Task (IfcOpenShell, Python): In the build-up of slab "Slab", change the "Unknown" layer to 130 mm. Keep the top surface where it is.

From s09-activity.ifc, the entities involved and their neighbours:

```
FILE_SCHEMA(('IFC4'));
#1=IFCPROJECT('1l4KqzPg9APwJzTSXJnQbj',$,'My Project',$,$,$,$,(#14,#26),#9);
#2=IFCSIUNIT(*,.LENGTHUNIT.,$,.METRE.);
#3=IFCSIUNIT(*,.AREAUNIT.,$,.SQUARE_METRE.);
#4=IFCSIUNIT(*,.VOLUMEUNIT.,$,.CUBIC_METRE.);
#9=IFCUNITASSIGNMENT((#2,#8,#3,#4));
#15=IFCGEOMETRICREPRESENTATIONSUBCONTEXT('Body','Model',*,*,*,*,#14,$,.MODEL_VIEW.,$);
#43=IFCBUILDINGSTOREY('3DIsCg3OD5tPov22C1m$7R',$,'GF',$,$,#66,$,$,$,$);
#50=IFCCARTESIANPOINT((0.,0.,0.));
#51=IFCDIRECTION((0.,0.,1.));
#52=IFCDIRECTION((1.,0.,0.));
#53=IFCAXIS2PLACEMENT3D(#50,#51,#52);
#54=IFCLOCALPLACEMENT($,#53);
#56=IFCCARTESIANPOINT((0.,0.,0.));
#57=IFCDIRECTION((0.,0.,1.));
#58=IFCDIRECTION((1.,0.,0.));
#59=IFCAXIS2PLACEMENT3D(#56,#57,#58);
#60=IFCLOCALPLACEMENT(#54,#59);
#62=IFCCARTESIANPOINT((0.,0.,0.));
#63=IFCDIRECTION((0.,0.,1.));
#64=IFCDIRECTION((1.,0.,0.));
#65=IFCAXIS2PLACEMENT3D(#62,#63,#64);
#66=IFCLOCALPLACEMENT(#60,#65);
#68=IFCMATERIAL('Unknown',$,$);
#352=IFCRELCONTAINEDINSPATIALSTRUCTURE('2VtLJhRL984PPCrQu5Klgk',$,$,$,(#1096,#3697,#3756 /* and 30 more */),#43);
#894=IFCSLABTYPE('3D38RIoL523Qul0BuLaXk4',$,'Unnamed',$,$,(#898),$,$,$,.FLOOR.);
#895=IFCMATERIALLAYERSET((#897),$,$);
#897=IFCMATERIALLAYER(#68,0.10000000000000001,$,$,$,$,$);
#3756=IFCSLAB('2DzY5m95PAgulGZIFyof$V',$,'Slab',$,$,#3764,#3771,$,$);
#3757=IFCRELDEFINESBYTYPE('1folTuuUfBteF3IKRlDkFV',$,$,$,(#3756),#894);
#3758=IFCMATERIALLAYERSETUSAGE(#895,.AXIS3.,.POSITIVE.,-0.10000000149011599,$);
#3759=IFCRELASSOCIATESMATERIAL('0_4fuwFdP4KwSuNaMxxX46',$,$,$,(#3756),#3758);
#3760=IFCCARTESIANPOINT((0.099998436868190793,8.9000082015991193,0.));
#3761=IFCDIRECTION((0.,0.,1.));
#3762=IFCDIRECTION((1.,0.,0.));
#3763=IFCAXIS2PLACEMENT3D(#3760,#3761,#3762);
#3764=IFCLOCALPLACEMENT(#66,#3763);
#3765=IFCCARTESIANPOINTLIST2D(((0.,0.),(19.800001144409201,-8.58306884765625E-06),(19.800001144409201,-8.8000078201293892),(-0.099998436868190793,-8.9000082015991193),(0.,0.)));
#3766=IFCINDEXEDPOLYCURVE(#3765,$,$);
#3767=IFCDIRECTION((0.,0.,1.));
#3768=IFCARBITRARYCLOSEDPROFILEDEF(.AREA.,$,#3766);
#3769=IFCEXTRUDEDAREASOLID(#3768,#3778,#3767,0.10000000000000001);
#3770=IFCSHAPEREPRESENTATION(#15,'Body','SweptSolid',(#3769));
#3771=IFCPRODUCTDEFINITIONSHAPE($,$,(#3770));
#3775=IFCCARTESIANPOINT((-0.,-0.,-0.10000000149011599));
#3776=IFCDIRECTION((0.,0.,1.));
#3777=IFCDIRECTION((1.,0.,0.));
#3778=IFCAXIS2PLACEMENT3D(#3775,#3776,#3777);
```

```python
import ifcopenshell
import ifcopenshell.util.element
import ifcopenshell.util.representation

model = ifcopenshell.open("s09-activity.ifc")

layer_set = model.by_id(895)
layer = next(l for l in layer_set.MaterialLayers if l.Material and l.Material.Name == "Unknown")
change = 0.13 - layer.LayerThickness
layer.LayerThickness += change

# Geometry does not follow the layer set by itself.
slabs = [e for e in ifcopenshell.util.element.get_elements_by_material(model, layer_set) if e.is_a("IfcSlab")]
for slab in sorted(slabs, key=lambda e: e.id()):
    body = ifcopenshell.util.representation.get_representation(slab, "Model", "Body")
    solid = body.Items[0]
    old_depth = solid.Depth
    solid.Depth += change
    # Extruded upwards: lower the start of the extrusion so the top stays.
    x, y, z = solid.Position.Location.Coordinates
    solid.Position.Location = model.createIfcCartesianPoint((x, y, z - change))
    print(slab.id(), f"{old_depth:g} -> {solid.Depth:g}")

# The layers are counted up from the underside, which has moved.
for usage in {ifcopenshell.util.element.get_material(slab) for slab in slabs}:
    usage.OffsetFromReferenceLine -= change

model.write("s09-activity-out.ifc")
```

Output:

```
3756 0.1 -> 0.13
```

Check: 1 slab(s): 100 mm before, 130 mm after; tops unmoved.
